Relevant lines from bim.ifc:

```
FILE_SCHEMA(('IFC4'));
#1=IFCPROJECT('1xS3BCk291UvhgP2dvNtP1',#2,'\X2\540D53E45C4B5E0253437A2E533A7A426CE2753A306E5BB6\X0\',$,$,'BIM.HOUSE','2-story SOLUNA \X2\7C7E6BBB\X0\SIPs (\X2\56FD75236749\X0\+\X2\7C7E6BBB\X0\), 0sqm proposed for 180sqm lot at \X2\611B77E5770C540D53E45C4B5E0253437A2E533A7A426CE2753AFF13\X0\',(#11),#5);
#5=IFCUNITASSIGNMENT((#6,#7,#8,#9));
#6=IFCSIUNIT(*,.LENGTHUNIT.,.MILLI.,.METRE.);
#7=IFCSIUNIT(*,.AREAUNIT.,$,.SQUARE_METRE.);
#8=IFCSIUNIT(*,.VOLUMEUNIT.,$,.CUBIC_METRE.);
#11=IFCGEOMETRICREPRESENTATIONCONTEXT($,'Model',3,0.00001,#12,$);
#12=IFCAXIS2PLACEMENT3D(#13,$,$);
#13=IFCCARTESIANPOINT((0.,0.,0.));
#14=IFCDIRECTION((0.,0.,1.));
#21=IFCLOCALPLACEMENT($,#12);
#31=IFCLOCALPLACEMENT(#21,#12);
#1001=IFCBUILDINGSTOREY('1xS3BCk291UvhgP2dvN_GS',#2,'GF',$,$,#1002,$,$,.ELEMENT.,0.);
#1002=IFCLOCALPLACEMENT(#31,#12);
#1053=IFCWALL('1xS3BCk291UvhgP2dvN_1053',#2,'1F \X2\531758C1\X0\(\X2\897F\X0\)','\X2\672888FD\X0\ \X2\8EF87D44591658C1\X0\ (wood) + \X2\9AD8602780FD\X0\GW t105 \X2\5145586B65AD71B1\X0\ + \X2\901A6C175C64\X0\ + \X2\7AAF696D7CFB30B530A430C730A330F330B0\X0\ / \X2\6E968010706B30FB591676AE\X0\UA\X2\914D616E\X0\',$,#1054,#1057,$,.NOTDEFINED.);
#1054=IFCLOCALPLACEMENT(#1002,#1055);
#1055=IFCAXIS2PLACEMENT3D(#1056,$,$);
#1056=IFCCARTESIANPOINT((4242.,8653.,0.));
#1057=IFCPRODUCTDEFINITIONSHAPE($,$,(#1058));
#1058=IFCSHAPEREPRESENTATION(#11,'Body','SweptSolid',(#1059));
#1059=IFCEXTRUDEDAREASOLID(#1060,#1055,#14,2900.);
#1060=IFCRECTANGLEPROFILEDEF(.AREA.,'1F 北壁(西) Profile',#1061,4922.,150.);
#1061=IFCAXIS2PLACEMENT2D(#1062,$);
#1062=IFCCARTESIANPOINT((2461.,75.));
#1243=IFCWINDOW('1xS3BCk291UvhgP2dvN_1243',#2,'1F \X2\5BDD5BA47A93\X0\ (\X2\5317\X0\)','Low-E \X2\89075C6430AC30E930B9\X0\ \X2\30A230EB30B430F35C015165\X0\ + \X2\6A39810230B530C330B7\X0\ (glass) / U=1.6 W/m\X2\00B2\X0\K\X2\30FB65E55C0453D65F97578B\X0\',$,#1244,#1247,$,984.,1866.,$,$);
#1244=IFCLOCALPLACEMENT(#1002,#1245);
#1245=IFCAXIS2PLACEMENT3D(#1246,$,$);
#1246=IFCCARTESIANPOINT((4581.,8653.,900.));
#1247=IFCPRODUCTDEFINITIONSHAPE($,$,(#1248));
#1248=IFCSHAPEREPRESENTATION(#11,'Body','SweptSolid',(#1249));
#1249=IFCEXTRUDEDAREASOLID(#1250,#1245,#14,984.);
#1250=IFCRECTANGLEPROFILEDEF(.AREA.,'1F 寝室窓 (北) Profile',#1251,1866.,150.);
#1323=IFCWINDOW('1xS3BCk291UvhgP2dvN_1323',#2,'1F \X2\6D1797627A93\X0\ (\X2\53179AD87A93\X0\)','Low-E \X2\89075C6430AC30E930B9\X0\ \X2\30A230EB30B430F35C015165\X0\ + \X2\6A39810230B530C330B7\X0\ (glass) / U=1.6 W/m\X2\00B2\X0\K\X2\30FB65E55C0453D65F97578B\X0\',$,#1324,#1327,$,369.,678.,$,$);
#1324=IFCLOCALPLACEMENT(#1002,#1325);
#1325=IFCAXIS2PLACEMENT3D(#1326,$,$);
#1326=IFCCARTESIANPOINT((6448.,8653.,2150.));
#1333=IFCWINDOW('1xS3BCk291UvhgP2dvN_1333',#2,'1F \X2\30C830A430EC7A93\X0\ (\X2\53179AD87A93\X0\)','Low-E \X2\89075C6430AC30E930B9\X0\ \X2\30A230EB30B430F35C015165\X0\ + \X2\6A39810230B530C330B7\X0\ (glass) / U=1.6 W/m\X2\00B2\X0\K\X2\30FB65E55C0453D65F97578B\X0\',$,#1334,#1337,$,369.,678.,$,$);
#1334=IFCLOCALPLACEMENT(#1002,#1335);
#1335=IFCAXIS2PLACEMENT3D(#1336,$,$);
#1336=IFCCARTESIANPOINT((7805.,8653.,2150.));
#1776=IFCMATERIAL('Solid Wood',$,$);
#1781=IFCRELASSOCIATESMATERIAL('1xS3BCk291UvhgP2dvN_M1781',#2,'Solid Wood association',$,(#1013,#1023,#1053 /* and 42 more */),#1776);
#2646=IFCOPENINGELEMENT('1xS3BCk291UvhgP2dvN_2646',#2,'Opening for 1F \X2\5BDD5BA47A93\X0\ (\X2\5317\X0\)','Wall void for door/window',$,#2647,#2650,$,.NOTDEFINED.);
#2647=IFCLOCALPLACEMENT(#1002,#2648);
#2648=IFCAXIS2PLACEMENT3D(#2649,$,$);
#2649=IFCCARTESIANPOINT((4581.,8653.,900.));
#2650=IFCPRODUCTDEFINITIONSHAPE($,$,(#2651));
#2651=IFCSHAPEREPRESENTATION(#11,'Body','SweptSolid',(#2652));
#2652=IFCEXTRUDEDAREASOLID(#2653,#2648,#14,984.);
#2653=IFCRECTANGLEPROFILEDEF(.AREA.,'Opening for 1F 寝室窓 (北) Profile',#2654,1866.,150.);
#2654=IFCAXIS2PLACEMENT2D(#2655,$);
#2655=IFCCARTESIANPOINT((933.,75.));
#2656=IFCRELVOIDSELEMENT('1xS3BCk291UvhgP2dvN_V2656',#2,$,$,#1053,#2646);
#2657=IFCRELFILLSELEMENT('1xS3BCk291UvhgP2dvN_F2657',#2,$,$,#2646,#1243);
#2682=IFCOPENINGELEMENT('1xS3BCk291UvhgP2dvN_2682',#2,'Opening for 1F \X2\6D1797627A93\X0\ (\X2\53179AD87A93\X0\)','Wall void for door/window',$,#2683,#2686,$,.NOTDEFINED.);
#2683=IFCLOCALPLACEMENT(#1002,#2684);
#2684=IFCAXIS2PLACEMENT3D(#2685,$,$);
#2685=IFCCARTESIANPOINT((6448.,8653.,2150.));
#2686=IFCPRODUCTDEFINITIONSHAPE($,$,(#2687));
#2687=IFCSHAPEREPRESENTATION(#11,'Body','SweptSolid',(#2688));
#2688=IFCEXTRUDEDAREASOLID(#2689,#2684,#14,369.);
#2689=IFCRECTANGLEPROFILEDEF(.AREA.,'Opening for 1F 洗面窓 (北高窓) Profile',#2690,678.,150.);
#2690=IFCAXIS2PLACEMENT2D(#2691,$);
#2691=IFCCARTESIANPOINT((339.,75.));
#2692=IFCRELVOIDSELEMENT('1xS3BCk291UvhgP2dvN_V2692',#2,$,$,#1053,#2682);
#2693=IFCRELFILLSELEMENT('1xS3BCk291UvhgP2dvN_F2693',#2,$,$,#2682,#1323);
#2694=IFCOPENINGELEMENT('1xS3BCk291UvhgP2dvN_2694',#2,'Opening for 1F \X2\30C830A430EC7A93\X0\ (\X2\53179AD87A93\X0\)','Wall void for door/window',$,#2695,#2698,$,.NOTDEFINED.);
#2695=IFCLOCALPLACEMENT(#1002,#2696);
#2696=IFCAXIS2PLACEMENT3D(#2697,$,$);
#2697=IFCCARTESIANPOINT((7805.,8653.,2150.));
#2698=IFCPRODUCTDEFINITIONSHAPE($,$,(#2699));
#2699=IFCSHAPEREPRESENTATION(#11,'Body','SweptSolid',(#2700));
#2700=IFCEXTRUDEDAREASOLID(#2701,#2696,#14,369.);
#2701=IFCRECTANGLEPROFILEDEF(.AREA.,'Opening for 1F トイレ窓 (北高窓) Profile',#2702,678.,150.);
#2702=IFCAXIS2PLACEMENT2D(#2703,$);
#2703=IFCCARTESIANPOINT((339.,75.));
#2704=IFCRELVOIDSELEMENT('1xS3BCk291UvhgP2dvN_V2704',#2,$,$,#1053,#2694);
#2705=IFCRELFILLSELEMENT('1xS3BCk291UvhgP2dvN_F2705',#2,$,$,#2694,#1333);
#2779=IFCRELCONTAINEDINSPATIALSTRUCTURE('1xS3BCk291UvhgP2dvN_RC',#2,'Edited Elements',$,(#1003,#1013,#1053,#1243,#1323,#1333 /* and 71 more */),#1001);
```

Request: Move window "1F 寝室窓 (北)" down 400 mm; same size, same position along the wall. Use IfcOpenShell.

```python
import numpy as np
import ifcopenshell
import ifcopenshell.api.geometry
import ifcopenshell.util.placement
import ifcopenshell.util.unit

model = ifcopenshell.open("bim.ifc")
unit_scale = ifcopenshell.util.unit.calculate_unit_scale(model)

window = model.by_guid("1xS3BCk291UvhgP2dvN_1243")
opening = window.FillsVoids[0].RelatingOpeningElement
dz = -0.4 / unit_scale

shift = np.array([0.0, 0.0, dz])
# The window is not placed relative to its opening, so move both.
for product in (opening, window):
    matrix = ifcopenshell.util.placement.get_local_placement(product.ObjectPlacement)
    matrix[:3, 3] += shift
    ifcopenshell.api.geometry.edit_object_placement(model, product=product, matrix=matrix, is_si=False)

print(f"moved by {dz * unit_scale:+.3f} m")

model.write("bim_rev.ifc")
```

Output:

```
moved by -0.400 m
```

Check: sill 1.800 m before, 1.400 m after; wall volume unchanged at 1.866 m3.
